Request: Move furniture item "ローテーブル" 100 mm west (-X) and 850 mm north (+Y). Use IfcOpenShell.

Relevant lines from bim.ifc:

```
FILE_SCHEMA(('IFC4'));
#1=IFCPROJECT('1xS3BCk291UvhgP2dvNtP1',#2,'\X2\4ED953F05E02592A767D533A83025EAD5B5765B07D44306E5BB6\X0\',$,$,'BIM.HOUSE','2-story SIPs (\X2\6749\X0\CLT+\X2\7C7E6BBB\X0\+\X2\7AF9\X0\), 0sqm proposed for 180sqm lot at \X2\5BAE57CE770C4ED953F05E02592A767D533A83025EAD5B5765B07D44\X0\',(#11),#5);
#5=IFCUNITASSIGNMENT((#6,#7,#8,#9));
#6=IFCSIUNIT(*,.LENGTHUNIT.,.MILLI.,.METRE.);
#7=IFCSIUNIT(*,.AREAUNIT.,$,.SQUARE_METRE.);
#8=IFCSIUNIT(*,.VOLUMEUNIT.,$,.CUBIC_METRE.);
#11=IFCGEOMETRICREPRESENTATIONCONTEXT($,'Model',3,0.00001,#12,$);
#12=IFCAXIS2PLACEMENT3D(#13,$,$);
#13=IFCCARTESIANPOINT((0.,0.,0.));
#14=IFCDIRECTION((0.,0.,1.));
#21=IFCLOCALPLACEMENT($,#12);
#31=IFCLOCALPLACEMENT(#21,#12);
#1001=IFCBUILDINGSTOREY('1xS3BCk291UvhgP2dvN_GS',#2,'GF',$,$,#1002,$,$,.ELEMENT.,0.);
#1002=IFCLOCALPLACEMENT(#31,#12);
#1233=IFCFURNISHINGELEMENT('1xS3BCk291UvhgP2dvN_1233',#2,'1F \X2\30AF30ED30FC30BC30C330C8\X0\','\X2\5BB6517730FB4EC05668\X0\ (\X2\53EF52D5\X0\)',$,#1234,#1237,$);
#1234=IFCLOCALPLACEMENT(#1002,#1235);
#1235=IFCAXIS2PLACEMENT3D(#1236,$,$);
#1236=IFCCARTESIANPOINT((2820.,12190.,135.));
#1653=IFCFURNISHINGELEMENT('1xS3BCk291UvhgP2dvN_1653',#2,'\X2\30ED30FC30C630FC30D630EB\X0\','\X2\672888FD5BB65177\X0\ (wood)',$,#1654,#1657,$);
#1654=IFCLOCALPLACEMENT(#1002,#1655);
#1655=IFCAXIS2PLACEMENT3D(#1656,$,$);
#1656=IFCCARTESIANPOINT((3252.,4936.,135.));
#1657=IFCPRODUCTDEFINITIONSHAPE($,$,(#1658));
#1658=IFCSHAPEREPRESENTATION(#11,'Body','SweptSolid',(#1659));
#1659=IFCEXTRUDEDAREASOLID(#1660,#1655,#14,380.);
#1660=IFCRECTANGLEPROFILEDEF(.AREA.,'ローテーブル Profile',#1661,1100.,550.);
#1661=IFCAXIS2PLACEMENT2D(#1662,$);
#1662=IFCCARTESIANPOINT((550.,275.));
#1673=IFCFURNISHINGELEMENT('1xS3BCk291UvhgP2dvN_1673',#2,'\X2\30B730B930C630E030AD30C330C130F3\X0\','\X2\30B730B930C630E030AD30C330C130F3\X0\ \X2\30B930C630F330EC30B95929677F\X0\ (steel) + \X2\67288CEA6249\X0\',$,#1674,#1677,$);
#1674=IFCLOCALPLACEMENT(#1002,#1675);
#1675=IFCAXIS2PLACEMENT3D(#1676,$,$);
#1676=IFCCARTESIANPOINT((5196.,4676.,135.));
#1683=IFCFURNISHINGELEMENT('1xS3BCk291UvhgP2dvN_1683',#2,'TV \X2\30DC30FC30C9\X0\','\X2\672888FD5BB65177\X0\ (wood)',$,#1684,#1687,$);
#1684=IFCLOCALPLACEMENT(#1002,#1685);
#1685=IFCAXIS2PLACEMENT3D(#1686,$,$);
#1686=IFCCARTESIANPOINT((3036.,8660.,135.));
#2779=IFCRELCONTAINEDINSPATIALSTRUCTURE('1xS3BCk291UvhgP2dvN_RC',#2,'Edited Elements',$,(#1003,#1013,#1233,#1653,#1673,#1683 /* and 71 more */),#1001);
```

```python
import ifcopenshell
import ifcopenshell.api.geometry
import ifcopenshell.util.placement
import ifcopenshell.util.unit

model = ifcopenshell.open("bim.ifc")
unit_scale = ifcopenshell.util.unit.calculate_unit_scale(model)

item = model.by_id(1653)
matrix = ifcopenshell.util.placement.get_local_placement(item.ObjectPlacement)
matrix[0, 3] -= 0.1 / unit_scale
matrix[1, 3] += 0.85 / unit_scale
ifcopenshell.api.geometry.edit_object_placement(model, product=item, matrix=matrix, is_si=False)

print(ifcopenshell.util.placement.get_local_placement(item.ObjectPlacement).round(3) + 0.0)

model.write("bim_edited.ifc")
```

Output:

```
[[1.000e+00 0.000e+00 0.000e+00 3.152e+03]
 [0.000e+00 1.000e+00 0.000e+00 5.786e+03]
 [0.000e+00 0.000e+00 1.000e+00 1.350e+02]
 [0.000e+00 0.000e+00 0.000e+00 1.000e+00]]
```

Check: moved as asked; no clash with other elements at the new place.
